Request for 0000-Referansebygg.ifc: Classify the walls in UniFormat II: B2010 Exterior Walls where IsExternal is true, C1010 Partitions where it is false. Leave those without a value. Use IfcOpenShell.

First a look at what the model holds.

```python
import ifcopenshell
import ifcopenshell.util.element

model = ifcopenshell.open("0000-Referansebygg.ifc")
print(model.schema)
print("classifications:", [c.Name for c in model.by_type("IfcClassification")])
values = [ifcopenshell.util.element.get_pset(e, "Pset_WallCommon", "IsExternal") for e in model.by_type("IfcWall")]
for value in (True, False, None):
    print("IsExternal", value, values.count(value))
```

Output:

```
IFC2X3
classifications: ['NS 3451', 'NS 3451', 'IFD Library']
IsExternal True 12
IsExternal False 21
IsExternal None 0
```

```python
import ifcopenshell
import ifcopenshell.api.classification
import ifcopenshell.util.element

model = ifcopenshell.open("0000-Referansebygg.ifc")

# IFC2X3 requires Source and Edition and has no link from the project to the system.
system = model.create_entity("IfcClassification", Source="ASTM", Edition="E1557", Name="UniFormat II")

walls = model.by_type("IfcWall")
external = {e: ifcopenshell.util.element.get_pset(e, "Pset_WallCommon", "IsExternal") for e in walls}
for flag, code, name in ((True, "B2010", "Exterior Walls"), (False, "C1010", "Partitions")):
    products = [e for e in walls if external[e] is flag]
    ifcopenshell.api.classification.add_reference(
        model, products=products, classification=system, identification=code, name=name
    )
    print(code, len(products))

model.write("0000-Referansebygg-out.ifc")
```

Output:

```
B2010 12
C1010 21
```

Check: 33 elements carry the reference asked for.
